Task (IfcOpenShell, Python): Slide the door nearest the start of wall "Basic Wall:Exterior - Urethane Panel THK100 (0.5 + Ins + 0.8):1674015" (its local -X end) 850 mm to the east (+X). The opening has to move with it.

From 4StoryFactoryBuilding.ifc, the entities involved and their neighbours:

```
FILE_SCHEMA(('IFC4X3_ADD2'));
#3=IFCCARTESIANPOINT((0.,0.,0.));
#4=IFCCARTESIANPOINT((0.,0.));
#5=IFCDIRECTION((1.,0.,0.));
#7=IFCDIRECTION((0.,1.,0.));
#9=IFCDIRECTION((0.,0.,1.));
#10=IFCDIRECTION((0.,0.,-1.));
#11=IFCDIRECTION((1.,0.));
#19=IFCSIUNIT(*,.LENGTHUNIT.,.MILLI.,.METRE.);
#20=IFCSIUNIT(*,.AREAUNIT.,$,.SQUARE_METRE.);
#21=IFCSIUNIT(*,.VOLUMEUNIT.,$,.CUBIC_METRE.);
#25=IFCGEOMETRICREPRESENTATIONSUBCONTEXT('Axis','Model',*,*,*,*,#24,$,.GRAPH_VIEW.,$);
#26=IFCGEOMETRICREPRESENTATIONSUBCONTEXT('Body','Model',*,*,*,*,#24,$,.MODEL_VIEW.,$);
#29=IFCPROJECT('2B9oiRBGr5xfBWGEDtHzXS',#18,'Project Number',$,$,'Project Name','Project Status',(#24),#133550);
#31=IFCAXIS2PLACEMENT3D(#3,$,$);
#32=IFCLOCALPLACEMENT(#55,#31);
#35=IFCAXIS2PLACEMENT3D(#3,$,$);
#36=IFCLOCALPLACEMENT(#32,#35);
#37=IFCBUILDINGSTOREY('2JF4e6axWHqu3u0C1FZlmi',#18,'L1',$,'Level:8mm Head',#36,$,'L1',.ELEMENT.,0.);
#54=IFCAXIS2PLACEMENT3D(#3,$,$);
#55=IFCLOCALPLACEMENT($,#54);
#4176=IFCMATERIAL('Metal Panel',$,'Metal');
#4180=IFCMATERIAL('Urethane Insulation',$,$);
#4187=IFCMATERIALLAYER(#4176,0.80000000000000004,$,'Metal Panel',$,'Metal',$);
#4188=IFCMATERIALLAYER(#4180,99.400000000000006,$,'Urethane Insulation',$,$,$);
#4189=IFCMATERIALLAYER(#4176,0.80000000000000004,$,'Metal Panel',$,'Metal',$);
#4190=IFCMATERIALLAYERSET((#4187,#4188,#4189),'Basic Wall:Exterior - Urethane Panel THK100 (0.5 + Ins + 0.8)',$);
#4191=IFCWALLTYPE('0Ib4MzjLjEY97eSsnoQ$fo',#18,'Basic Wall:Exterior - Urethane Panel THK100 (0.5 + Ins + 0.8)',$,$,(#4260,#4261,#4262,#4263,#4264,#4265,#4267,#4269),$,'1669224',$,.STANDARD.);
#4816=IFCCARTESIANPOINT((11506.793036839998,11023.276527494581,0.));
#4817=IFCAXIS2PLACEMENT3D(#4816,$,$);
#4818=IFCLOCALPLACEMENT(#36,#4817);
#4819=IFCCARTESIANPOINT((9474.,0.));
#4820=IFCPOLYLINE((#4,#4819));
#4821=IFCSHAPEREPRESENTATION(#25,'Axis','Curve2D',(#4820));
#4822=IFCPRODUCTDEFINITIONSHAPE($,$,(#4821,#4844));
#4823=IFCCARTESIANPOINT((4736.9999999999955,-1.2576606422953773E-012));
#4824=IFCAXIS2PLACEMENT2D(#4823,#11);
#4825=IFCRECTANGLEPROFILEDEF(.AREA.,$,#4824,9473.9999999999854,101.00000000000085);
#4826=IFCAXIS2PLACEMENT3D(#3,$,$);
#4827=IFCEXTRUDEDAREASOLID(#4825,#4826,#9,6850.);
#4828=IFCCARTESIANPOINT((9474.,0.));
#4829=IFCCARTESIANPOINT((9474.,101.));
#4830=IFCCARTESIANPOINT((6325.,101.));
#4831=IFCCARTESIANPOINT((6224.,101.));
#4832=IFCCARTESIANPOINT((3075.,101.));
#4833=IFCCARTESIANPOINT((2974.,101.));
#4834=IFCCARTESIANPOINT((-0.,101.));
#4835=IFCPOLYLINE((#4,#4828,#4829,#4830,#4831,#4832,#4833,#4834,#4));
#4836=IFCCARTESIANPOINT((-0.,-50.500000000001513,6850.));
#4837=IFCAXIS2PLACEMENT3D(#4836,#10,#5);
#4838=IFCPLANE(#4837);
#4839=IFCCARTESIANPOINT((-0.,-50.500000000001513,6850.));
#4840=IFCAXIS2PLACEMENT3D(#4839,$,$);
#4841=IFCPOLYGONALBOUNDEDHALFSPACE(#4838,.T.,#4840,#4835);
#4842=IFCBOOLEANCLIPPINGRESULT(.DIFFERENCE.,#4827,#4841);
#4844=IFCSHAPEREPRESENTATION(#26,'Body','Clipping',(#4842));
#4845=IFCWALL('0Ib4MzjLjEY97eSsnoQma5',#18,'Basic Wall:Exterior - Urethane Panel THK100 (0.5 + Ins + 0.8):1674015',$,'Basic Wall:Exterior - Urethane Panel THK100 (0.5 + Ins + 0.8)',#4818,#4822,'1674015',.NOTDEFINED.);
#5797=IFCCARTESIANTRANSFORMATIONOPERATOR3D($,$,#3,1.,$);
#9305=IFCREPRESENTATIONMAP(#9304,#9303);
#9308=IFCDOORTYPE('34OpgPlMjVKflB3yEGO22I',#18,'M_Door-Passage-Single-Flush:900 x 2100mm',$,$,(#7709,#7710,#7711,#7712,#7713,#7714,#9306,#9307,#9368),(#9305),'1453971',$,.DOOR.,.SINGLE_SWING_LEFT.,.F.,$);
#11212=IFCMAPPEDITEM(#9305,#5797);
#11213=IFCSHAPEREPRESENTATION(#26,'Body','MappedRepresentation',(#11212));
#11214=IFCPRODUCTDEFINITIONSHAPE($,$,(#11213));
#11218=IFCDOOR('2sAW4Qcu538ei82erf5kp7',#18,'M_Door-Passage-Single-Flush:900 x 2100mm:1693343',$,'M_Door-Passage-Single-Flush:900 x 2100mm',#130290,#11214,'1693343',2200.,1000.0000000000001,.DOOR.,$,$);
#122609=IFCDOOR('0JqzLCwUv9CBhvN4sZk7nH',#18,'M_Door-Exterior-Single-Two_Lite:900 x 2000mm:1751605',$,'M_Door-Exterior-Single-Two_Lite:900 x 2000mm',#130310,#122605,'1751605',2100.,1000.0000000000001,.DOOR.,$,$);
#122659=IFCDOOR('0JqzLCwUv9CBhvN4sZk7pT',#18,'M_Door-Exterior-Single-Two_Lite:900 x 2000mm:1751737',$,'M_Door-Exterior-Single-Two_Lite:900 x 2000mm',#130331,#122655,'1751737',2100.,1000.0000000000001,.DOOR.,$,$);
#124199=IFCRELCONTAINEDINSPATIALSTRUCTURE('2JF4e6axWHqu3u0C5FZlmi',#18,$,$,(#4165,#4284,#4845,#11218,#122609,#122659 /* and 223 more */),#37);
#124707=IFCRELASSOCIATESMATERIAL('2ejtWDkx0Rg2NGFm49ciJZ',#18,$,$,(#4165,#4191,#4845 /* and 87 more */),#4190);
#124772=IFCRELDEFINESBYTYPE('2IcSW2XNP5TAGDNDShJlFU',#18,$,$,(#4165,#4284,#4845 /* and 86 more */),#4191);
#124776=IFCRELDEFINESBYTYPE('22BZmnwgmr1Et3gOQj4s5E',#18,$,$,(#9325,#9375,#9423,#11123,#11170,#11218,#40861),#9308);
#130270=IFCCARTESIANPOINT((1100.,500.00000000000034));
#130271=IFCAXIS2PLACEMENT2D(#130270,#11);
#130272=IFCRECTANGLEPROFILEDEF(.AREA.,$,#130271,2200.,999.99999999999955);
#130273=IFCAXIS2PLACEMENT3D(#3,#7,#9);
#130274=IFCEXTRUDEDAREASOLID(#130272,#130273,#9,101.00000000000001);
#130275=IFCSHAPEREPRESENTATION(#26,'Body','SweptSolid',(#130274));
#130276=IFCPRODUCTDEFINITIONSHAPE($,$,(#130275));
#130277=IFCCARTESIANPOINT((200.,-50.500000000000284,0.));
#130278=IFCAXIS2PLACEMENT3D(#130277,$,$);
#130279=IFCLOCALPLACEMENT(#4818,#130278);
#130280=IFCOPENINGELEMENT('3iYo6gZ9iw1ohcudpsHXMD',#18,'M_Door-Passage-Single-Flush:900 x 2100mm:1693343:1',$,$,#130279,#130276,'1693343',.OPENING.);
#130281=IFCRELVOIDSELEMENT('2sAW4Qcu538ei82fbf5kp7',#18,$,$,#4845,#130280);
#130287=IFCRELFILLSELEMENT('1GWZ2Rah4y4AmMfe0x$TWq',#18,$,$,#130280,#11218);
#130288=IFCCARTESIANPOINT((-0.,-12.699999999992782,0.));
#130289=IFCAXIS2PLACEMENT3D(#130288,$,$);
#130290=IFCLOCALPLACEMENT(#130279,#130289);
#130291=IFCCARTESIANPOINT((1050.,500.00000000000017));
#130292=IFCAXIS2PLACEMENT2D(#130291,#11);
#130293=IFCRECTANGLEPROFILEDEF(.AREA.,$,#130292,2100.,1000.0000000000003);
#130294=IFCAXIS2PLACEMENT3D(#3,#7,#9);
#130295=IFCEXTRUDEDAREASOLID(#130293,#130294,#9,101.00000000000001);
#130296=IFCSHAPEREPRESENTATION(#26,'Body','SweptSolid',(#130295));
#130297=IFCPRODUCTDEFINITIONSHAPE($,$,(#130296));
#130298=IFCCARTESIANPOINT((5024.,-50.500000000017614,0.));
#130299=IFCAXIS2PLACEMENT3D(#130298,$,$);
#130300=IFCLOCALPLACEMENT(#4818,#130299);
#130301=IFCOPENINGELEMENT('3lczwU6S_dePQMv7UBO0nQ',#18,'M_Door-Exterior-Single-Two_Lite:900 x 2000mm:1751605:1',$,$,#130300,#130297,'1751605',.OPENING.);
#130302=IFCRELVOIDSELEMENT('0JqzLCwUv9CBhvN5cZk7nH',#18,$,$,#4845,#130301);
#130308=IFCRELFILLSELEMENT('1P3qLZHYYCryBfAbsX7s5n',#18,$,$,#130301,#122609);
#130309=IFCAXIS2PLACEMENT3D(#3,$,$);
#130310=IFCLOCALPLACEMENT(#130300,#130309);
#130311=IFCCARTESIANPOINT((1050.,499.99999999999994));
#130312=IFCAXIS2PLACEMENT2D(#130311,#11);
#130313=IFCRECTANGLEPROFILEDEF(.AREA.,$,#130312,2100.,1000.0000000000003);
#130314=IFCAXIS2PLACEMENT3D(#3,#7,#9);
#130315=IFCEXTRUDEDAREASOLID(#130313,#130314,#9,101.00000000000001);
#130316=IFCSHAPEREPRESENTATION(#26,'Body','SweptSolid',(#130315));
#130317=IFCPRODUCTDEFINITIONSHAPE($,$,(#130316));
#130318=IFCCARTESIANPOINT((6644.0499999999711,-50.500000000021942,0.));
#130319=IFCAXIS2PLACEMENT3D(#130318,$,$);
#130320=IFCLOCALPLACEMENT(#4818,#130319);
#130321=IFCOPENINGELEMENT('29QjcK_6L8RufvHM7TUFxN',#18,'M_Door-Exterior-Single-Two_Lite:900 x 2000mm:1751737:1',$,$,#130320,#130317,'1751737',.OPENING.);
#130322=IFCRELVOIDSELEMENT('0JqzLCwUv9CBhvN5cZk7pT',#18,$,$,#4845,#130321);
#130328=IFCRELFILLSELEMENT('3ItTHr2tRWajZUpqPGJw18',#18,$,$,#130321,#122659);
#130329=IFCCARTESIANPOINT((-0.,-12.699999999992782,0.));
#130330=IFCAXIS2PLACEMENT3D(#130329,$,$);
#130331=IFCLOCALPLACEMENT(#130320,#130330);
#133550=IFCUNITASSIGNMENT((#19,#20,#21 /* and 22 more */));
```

```python
import ifcopenshell
import ifcopenshell.api.geometry
import ifcopenshell.util.placement
import ifcopenshell.util.unit

model = ifcopenshell.open("4StoryFactoryBuilding.ifc")
unit_scale = ifcopenshell.util.unit.calculate_unit_scale(model)

door = model.by_guid("2sAW4Qcu538ei82erf5kp7")
opening = door.FillsVoids[0].RelatingOpeningElement
wall = opening.VoidsElements[0].RelatingBuildingElement

wall_matrix = ifcopenshell.util.placement.get_local_placement(wall.ObjectPlacement)
shift = wall_matrix[:3, 0] * 0.85 / unit_scale
before = ifcopenshell.util.placement.get_local_placement(door.ObjectPlacement)[:3, 3].copy()

# The door is placed relative to its opening, so it follows when the opening moves.
matrix = ifcopenshell.util.placement.get_local_placement(opening.ObjectPlacement)
matrix[:3, 3] += shift
ifcopenshell.api.geometry.edit_object_placement(
    model, product=opening, matrix=matrix, is_si=False, should_transform_children=True
)

after = ifcopenshell.util.placement.get_local_placement(door.ObjectPlacement)[:3, 3]
print("door moved by", (after - before).round(3) + 0.0)

model.write("4StoryFactoryBuilding_edited.ifc")
```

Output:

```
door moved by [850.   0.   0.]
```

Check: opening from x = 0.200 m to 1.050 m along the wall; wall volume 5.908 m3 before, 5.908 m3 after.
